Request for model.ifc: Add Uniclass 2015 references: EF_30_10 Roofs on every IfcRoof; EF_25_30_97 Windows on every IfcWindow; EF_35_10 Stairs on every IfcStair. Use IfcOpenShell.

First a look at what the model holds.

```python
import ifcopenshell

model = ifcopenshell.open("model.ifc")
print(model.schema)
print("classifications:", [c.Name for c in model.by_type("IfcClassification")])
for ifc_class in ("IfcDoor", "IfcRoof", "IfcStair", "IfcWall", "IfcWindow"):
    print(ifc_class, len(model.by_type(ifc_class)))
```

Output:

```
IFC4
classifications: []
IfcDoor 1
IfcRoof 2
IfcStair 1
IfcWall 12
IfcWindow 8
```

```python
import ifcopenshell
import ifcopenshell.api.classification

model = ifcopenshell.open("model.ifc")

system = ifcopenshell.api.classification.add_classification(model, classification="Uniclass 2015")

codes = {
    "IfcRoof": ("EF_30_10", "Roofs"),
    "IfcWindow": ("EF_25_30_97", "Windows"),
    "IfcStair": ("EF_35_10", "Stairs"),
}
for ifc_class, (code, name) in codes.items():
    products = model.by_type(ifc_class)
    ifcopenshell.api.classification.add_reference(
        model, products=products, classification=system, identification=code, name=name
    )
    print(code, len(products))

model.write("model-out.ifc")
```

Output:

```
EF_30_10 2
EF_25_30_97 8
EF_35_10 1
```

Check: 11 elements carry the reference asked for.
